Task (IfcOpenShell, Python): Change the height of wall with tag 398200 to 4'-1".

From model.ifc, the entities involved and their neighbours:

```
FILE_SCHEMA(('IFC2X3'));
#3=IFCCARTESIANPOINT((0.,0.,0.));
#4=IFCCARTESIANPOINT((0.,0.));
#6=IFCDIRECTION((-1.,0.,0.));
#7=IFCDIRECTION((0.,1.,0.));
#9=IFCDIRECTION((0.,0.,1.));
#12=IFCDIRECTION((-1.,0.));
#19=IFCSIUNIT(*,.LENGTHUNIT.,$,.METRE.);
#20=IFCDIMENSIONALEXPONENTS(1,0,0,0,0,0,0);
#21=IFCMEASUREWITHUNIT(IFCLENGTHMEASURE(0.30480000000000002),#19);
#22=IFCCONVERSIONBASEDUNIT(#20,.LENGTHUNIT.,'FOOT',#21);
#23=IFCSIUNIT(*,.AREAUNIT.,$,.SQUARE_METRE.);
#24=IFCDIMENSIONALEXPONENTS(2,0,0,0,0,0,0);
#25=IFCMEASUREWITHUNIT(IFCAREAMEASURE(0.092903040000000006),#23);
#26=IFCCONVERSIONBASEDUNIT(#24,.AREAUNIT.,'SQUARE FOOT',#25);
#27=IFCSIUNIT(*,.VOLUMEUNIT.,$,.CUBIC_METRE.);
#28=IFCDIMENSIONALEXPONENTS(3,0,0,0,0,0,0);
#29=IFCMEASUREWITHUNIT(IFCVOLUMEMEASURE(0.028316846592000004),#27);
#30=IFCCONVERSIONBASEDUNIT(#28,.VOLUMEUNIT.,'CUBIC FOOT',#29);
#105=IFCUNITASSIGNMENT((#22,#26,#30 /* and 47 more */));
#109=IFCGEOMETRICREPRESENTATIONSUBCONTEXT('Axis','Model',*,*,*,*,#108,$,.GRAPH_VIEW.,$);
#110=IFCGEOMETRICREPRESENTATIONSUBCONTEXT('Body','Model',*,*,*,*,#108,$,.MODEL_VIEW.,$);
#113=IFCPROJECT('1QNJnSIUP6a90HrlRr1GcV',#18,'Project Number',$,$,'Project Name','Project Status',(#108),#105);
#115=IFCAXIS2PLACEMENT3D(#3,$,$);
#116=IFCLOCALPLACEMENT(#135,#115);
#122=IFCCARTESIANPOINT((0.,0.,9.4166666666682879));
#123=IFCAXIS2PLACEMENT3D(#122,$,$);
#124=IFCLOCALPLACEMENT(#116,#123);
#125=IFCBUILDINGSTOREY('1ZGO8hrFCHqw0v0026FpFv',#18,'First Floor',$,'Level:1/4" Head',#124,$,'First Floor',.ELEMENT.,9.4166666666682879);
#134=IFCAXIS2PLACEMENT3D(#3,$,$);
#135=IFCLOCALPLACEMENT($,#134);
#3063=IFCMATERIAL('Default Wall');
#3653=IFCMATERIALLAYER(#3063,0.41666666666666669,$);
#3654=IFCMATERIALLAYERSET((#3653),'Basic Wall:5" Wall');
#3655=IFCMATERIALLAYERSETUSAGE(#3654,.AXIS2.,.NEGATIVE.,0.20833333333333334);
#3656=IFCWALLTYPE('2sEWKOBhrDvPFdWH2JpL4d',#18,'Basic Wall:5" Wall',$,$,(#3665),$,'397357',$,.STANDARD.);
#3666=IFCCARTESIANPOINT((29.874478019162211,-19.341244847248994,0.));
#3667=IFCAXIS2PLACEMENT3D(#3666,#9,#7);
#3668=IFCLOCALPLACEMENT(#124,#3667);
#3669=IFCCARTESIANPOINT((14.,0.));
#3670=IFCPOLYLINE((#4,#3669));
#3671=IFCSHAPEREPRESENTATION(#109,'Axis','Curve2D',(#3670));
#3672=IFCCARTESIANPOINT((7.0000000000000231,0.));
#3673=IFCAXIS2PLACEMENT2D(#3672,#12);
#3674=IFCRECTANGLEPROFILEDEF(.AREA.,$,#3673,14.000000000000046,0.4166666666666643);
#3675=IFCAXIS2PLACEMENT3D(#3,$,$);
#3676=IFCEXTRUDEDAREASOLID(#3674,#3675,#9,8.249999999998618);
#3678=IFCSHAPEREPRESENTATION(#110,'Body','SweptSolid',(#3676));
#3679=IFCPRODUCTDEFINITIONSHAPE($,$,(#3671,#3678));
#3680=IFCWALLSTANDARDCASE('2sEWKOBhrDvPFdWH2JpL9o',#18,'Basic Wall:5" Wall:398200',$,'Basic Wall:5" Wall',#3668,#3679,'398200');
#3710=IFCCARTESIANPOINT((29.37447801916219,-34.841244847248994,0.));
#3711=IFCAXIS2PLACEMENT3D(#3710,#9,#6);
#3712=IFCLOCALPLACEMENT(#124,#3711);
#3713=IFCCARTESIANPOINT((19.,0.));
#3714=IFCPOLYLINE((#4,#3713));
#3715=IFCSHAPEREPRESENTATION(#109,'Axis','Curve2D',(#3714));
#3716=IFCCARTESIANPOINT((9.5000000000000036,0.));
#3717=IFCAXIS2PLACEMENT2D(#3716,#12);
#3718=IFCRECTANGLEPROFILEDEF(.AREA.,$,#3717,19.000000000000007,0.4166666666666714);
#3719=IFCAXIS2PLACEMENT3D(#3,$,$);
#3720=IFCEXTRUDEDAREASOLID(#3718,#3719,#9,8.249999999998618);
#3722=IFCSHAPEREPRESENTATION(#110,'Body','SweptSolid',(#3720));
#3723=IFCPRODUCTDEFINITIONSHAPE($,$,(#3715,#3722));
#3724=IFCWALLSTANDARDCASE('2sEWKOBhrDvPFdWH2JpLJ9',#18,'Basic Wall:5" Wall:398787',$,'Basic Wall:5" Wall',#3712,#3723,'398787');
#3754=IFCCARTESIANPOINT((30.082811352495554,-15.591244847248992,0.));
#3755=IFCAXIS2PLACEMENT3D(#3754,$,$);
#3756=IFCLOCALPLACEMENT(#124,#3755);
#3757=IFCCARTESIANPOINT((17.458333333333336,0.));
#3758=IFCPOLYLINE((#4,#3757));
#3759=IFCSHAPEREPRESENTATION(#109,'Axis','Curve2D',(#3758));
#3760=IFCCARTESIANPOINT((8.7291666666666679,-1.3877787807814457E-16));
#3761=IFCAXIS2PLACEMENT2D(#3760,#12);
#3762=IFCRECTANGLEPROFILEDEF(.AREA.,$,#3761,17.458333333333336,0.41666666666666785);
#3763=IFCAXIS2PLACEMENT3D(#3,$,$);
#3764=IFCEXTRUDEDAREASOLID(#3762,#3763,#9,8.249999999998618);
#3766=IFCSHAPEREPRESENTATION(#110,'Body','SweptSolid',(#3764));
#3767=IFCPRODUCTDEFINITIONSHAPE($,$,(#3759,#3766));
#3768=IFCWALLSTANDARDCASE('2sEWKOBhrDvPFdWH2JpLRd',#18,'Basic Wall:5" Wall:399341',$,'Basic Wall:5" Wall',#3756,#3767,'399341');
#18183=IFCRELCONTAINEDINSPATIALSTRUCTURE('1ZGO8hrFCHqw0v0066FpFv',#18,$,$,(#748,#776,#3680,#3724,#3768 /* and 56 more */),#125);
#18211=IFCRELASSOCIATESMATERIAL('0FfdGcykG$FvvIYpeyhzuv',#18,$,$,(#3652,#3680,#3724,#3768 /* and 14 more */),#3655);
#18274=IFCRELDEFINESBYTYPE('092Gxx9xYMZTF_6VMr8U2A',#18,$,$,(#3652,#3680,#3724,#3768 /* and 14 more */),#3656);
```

```python
import ifcopenshell
import ifcopenshell.geom
import ifcopenshell.util.representation
import ifcopenshell.util.shape
import ifcopenshell.util.unit

model = ifcopenshell.open("model.ifc")
unit_scale = ifcopenshell.util.unit.calculate_unit_scale(model)
settings = ifcopenshell.geom.settings()


def volume(element):
    """Net volume in cubic metres, openings subtracted."""
    shape = ifcopenshell.geom.create_shape(settings, element)
    return ifcopenshell.util.shape.get_volume(shape.geometry)


wall = model.by_guid("2sEWKOBhrDvPFdWH2JpL9o")
before = volume(wall)

body = ifcopenshell.util.representation.get_representation(wall, "Model", "Body")
solid = body.Items[0]
old_height = solid.Depth
solid.Depth = 49 * 0.0254 / unit_scale
after = volume(wall)

print(f"height {old_height:g} -> {solid.Depth:g}, volume {before:.3f} -> {after:.3f} m3")

model.write("model_updated.ifc")
```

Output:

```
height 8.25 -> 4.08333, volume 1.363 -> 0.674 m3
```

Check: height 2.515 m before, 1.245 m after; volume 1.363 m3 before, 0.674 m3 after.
